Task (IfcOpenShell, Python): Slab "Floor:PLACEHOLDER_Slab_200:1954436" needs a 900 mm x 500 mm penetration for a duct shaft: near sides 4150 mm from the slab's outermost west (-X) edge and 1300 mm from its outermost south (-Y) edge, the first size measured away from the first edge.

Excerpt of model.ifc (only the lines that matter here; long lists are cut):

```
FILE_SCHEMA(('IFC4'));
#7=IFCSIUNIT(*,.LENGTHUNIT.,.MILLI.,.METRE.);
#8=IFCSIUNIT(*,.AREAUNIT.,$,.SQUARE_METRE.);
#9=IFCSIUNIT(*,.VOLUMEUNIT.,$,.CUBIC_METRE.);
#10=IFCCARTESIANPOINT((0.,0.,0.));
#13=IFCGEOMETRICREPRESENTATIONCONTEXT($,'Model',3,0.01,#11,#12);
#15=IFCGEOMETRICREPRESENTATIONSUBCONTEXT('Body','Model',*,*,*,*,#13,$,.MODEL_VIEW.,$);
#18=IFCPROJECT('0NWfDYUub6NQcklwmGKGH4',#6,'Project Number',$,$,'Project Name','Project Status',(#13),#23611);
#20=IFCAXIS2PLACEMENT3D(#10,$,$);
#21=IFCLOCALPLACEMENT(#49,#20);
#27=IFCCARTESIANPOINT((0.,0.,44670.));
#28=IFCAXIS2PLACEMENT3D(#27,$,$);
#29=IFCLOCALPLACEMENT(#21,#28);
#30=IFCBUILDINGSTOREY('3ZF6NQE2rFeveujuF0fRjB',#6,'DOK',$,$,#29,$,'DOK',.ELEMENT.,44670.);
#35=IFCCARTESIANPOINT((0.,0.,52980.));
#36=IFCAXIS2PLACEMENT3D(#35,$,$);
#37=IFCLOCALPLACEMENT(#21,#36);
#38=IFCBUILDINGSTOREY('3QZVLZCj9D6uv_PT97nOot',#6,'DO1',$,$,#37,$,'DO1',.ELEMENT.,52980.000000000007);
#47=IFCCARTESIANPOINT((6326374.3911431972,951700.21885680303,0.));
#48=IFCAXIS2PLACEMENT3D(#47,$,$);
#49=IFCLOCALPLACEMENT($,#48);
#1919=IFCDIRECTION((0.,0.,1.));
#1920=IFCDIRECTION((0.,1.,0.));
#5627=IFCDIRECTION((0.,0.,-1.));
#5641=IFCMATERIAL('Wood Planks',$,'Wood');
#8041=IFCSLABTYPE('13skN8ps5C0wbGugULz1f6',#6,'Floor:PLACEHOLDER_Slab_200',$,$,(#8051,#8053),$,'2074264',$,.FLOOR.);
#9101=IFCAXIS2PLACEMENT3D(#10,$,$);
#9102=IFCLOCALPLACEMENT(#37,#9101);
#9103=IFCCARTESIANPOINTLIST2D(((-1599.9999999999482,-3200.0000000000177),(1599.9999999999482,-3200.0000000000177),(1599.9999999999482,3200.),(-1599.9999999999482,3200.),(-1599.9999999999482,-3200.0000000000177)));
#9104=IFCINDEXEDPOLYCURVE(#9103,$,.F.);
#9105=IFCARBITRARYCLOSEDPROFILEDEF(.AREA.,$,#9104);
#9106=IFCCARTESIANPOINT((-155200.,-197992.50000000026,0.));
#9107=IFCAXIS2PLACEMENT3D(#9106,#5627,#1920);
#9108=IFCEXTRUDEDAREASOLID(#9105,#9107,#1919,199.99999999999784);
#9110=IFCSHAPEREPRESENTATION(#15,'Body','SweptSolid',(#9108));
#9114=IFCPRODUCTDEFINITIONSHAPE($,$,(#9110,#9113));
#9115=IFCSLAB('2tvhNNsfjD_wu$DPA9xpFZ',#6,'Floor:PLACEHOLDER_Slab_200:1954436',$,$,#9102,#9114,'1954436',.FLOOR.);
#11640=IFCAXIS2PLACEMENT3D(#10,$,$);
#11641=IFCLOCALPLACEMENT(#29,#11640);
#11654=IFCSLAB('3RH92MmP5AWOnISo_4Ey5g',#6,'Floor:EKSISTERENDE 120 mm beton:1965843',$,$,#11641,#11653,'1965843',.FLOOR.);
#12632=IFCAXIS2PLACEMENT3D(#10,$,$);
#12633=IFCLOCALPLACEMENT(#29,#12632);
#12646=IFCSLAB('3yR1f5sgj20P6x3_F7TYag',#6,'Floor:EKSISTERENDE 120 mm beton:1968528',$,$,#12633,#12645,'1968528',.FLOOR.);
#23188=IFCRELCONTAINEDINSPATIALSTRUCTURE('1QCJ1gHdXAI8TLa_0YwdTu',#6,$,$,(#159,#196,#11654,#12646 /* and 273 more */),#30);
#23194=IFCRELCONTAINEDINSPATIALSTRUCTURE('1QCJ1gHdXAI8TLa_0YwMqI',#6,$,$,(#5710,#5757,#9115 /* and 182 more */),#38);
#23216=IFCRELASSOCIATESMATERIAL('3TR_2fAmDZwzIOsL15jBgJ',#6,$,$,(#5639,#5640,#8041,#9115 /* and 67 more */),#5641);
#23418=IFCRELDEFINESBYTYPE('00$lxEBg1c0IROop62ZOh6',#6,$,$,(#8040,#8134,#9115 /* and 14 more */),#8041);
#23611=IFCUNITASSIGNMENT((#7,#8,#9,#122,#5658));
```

```python
import numpy as np
import ifcopenshell
import ifcopenshell.api.feature
import ifcopenshell.api.geometry
import ifcopenshell.api.root
import ifcopenshell.geom
import ifcopenshell.util.placement
import ifcopenshell.util.representation
import ifcopenshell.util.shape
import ifcopenshell.util.unit

model = ifcopenshell.open("model.ifc")
unit_scale = ifcopenshell.util.unit.calculate_unit_scale(model)
settings = ifcopenshell.geom.settings()


def volume(element):
    """Net volume in cubic metres, openings subtracted."""
    shape = ifcopenshell.geom.create_shape(settings, element)
    return ifcopenshell.util.shape.get_volume(shape.geometry)


slab = model.by_guid("2tvhNNsfjD_wu$DPA9xpFZ")
before = volume(slab)

# Extent in the slab's own axes, in metres. The edges named are its -X and -Y sides.
slab_shape = ifcopenshell.geom.create_shape(settings, slab)
vertices = ifcopenshell.util.shape.get_vertices(slab_shape.geometry)
x_min, y_min, bottom = vertices.min(axis=0)
top = vertices[:, 2].max()

opening = ifcopenshell.api.root.create_entity(model, ifc_class="IfcOpeningElement", name="Duct shaft opening", predefined_type="OPENING")
context = ifcopenshell.util.representation.get_context(model, "Model", "Body", "MODEL_VIEW")
width, depth = 0.9, 0.5
outline = [(0.0, 0.0), (width, 0.0), (width, depth), (0.0, depth), (0.0, 0.0)]
# Overshoot both faces by 50 mm so the cut is clean.
shape = ifcopenshell.api.geometry.add_slab_representation(
    model, context=context, depth=top - bottom + 0.1, polyline=outline
)
ifcopenshell.api.geometry.assign_representation(model, product=opening, representation=shape)

matrix = ifcopenshell.util.placement.get_local_placement(slab.ObjectPlacement)
matrix[:, 3] = matrix @ np.append(np.array([x_min + 4.15, y_min + 1.3, bottom - 0.05]) / unit_scale, 1.0)
ifcopenshell.api.geometry.edit_object_placement(model, product=opening, matrix=matrix, is_si=False)
ifcopenshell.api.feature.add_feature(model, feature=opening, element=slab)

after = volume(slab)

print(f"slab volume {before:.3f} -> {after:.3f} m3")

model.write("model-out.ifc")
```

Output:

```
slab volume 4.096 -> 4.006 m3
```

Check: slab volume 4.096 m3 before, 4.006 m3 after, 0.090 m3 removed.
